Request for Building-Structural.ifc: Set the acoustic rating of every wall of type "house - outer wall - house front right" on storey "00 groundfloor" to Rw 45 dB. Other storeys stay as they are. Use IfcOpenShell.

First a look at what the model holds.

```python
import ifcopenshell
import ifcopenshell.util.element

model = ifcopenshell.open("Building-Structural.ifc")
print(model.schema)
storey = next(s for s in model.by_type("IfcBuildingStorey") if s.Name == "00 groundfloor")
walls = [e for e in ifcopenshell.util.element.get_decomposition(storey) if e.is_a("IfcWall")]
seen = {}
for e in walls:
    element_type = ifcopenshell.util.element.get_type(e)
    key = (element_type.Name if element_type != e and element_type else None, ifcopenshell.util.element.get_pset(e, "Pset_WallCommon", "AcousticRating"))
    seen[key] = seen.get(key, 0) + 1
for (name, value), count in sorted(seen.items(), key=str):
    print(count, "x", name, "|", value)
```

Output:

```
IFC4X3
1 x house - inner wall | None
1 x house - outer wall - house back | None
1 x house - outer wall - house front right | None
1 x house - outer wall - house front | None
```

```python
import ifcopenshell
import ifcopenshell.api.pset
import ifcopenshell.util.element

model = ifcopenshell.open("Building-Structural.ifc")

storey = next(s for s in model.by_type("IfcBuildingStorey") if s.Name == "00 groundfloor")
walls = [e for e in ifcopenshell.util.element.get_decomposition(storey) if e.is_a("IfcWall")]

count = 0
for e in walls:
    element_type = ifcopenshell.util.element.get_type(e)
    if element_type in (None, e) or element_type.Name != "house - outer wall - house front right":
        continue
    # add_pset returns the element's existing set when there is one.
    pset = ifcopenshell.api.pset.add_pset(model, product=e, name="Pset_WallCommon")
    ifcopenshell.api.pset.edit_pset(model, pset=pset, properties={"AcousticRating": "Rw 45 dB"})
    count += 1

print(count, "walls updated")

model.write("Building-Structural_rev.ifc")
```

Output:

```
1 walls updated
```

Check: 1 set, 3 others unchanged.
